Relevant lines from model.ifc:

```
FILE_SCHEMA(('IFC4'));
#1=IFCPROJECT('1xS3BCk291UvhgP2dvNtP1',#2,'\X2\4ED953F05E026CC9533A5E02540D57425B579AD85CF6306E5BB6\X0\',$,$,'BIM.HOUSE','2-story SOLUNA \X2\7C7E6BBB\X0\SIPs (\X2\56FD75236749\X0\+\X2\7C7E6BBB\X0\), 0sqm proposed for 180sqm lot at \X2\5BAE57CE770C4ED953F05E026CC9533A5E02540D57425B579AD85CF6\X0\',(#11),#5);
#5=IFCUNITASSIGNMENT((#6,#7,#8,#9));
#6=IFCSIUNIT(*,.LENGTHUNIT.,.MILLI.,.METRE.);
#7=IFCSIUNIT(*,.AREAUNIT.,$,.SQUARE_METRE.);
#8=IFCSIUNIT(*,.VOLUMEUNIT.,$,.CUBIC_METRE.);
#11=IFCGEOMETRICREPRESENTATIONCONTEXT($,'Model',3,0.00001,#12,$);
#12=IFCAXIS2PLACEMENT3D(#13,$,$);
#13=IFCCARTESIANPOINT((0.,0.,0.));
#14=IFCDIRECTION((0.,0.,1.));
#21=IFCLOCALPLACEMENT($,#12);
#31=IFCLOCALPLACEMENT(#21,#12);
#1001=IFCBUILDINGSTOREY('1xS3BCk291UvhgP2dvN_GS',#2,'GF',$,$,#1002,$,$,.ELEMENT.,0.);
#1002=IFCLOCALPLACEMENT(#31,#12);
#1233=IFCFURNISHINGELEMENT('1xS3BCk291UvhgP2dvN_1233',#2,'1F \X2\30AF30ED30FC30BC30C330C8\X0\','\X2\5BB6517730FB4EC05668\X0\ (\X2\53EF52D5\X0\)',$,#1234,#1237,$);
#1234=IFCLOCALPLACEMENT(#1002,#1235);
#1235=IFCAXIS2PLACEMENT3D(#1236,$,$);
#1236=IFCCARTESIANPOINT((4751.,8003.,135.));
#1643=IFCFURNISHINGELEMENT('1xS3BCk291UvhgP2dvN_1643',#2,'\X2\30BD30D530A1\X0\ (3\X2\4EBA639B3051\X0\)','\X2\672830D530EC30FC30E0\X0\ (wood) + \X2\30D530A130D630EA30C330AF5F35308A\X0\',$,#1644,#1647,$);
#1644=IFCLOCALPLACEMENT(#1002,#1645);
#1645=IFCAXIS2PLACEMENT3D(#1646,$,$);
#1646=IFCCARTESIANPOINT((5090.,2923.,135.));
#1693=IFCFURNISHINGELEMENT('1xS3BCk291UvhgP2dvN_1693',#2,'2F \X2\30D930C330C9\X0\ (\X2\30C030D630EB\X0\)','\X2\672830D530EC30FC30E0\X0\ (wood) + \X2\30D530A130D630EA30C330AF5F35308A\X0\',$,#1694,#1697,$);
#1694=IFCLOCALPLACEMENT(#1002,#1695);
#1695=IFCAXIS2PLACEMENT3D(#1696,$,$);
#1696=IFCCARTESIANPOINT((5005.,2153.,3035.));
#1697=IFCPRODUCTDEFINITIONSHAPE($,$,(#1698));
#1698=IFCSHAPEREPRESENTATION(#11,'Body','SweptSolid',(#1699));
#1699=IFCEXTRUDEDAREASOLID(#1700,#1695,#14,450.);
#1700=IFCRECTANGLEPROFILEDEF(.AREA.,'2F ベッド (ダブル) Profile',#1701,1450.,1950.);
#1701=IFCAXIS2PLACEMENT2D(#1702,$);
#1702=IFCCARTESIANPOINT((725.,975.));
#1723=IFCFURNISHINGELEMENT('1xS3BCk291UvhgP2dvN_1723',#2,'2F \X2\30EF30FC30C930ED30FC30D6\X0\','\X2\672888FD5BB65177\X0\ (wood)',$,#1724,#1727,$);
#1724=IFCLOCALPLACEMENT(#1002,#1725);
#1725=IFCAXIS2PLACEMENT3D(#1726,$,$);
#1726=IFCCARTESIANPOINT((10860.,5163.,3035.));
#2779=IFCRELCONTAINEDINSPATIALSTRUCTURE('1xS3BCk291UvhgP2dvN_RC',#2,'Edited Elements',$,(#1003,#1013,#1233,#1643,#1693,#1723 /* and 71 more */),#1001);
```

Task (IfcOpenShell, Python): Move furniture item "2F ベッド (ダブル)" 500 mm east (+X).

```python
import ifcopenshell
import ifcopenshell.api.geometry
import ifcopenshell.util.placement
import ifcopenshell.util.unit

model = ifcopenshell.open("model.ifc")
unit_scale = ifcopenshell.util.unit.calculate_unit_scale(model)

item = model.by_id(1693)
matrix = ifcopenshell.util.placement.get_local_placement(item.ObjectPlacement)
matrix[0, 3] += 0.5 / unit_scale
ifcopenshell.api.geometry.edit_object_placement(model, product=item, matrix=matrix, is_si=False)

print(ifcopenshell.util.placement.get_local_placement(item.ObjectPlacement).round(3) + 0.0)

model.write("model_rev.ifc")
```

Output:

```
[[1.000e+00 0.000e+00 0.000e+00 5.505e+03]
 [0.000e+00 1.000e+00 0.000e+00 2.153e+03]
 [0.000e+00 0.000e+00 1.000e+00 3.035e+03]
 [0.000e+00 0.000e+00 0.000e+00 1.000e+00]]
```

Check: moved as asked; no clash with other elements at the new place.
